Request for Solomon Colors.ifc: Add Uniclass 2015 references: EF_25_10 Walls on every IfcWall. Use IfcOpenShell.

First a look at what the model holds.

```python
import ifcopenshell

model = ifcopenshell.open("Solomon Colors.ifc")
print(model.schema)
print("classifications:", [c.Name for c in model.by_type("IfcClassification")])
for ifc_class in ("IfcDoor", "IfcRoof", "IfcStair", "IfcWall", "IfcWindow"):
    print(ifc_class, len(model.by_type(ifc_class)))
```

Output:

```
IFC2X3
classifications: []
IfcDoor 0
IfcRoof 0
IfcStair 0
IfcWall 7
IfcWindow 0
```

```python
import ifcopenshell
import ifcopenshell.api.classification

model = ifcopenshell.open("Solomon Colors.ifc")

# IFC2X3 requires Source and Edition and has no link from the project to the system.
system = model.create_entity("IfcClassification", Source="NBS", Edition="2015", Name="Uniclass 2015")

codes = {
    "IfcWall": ("EF_25_10", "Walls"),
}
for ifc_class, (code, name) in codes.items():
    products = model.by_type(ifc_class)
    ifcopenshell.api.classification.add_reference(
        model, products=products, classification=system, identification=code, name=name
    )
    print(code, len(products))

model.write("Solomon Colors_v2.ifc")
```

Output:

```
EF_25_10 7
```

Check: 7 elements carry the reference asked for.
